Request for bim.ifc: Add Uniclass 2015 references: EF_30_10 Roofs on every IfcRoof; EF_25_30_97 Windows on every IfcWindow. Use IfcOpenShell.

First a look at what the model holds.

```python
import ifcopenshell

model = ifcopenshell.open("bim.ifc")
print(model.schema)
print("classifications:", [c.Name for c in model.by_type("IfcClassification")])
for ifc_class in ("IfcDoor", "IfcRoof", "IfcStair", "IfcWall", "IfcWindow"):
    print(ifc_class, len(model.by_type(ifc_class)))
```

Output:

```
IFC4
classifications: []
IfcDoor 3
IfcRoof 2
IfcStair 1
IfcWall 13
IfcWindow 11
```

```python
import ifcopenshell
import ifcopenshell.api.classification

model = ifcopenshell.open("bim.ifc")

system = ifcopenshell.api.classification.add_classification(model, classification="Uniclass 2015")

codes = {
    "IfcRoof": ("EF_30_10", "Roofs"),
    "IfcWindow": ("EF_25_30_97", "Windows"),
}
for ifc_class, (code, name) in codes.items():
    products = model.by_type(ifc_class)
    ifcopenshell.api.classification.add_reference(
        model, products=products, classification=system, identification=code, name=name
    )
    print(code, len(products))

model.write("bim_edited.ifc")
```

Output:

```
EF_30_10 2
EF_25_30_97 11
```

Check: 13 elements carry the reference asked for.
